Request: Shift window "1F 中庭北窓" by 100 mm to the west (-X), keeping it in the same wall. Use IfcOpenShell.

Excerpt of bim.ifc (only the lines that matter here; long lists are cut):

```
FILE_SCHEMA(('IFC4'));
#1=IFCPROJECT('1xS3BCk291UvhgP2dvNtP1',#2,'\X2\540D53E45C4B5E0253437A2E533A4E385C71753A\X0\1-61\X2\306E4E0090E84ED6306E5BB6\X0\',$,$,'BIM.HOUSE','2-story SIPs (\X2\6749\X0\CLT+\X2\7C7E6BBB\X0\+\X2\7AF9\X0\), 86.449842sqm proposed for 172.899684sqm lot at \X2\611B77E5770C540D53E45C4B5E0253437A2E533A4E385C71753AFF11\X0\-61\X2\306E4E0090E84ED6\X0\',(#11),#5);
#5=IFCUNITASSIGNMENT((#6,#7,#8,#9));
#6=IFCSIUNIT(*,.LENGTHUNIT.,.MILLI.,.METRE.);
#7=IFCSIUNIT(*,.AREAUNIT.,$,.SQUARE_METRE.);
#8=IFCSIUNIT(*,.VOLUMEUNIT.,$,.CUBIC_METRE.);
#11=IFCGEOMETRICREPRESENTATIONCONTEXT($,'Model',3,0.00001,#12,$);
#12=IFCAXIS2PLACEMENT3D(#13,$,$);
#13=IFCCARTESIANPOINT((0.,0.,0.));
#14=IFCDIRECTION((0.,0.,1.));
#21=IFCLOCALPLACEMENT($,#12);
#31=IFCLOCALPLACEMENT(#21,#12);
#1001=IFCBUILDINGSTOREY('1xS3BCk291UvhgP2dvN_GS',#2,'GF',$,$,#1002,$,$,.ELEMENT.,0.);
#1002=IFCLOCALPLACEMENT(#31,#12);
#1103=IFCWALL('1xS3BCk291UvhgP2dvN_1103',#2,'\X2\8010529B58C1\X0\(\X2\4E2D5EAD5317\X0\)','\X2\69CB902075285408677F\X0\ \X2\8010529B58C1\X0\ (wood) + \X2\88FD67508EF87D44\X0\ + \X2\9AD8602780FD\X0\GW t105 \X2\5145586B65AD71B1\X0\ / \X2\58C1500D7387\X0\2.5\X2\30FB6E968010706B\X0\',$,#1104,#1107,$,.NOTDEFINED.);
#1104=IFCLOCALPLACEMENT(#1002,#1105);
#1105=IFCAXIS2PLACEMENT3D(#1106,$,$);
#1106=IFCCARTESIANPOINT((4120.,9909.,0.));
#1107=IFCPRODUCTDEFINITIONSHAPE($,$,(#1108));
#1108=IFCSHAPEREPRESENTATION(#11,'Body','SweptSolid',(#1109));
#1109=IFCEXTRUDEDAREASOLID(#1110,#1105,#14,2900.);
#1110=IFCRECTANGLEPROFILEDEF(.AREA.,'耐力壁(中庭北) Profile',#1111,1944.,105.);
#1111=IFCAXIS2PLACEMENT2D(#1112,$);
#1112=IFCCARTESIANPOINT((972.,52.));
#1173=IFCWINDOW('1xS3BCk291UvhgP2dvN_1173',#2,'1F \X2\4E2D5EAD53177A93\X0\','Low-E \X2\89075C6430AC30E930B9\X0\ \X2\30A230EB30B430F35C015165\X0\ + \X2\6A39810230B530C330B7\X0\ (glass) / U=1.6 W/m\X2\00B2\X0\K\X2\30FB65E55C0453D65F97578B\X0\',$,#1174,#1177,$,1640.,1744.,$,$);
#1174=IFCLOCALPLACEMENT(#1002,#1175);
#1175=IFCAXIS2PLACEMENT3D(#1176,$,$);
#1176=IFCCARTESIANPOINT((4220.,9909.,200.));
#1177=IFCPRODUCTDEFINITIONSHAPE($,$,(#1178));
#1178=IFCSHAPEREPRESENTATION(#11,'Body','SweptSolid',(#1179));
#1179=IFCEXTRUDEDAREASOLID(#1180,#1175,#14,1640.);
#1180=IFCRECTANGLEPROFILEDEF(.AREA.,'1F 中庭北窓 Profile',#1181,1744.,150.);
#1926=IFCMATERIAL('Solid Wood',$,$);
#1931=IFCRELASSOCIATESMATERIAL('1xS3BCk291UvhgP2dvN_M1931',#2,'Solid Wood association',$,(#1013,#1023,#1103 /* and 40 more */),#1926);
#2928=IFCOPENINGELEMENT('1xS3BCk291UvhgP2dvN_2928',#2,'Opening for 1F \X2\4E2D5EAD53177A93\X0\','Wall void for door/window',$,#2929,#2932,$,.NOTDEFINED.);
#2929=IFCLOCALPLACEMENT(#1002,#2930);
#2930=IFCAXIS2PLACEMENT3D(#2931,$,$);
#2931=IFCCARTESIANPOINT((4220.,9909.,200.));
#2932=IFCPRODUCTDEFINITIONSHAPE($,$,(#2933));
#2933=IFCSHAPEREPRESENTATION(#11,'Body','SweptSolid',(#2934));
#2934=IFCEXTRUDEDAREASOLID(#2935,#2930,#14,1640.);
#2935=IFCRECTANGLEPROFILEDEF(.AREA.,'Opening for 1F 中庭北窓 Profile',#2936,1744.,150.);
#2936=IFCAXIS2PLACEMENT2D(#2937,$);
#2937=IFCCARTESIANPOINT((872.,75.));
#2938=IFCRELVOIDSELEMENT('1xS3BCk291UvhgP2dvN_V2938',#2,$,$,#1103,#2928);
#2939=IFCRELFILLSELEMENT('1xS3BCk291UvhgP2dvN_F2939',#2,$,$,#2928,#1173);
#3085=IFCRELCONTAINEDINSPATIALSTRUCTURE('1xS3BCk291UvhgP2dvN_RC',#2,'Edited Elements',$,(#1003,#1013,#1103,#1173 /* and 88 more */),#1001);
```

```python
import ifcopenshell
import ifcopenshell.api.geometry
import ifcopenshell.util.placement

model = ifcopenshell.open("bim.ifc")

window = model.by_id(1173)
opening = window.FillsVoids[0].RelatingOpeningElement
wall = opening.VoidsElements[0].RelatingBuildingElement

wall_matrix = ifcopenshell.util.placement.get_local_placement(wall.ObjectPlacement)
shift = wall_matrix[:3, 0] * -100.0
before = ifcopenshell.util.placement.get_local_placement(window.ObjectPlacement)[:3, 3].copy()

# The window is not placed relative to its opening, so move both.
for product in (opening, window):
    matrix = ifcopenshell.util.placement.get_local_placement(product.ObjectPlacement)
    matrix[:3, 3] += shift
    ifcopenshell.api.geometry.edit_object_placement(model, product=product, matrix=matrix, is_si=False)

after = ifcopenshell.util.placement.get_local_placement(window.ObjectPlacement)[:3, 3]
print("window moved by", (after - before).round(3) + 0.0)

model.write("bim-out.ifc")
```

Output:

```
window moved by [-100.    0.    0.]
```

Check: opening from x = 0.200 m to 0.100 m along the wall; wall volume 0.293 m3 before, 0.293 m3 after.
